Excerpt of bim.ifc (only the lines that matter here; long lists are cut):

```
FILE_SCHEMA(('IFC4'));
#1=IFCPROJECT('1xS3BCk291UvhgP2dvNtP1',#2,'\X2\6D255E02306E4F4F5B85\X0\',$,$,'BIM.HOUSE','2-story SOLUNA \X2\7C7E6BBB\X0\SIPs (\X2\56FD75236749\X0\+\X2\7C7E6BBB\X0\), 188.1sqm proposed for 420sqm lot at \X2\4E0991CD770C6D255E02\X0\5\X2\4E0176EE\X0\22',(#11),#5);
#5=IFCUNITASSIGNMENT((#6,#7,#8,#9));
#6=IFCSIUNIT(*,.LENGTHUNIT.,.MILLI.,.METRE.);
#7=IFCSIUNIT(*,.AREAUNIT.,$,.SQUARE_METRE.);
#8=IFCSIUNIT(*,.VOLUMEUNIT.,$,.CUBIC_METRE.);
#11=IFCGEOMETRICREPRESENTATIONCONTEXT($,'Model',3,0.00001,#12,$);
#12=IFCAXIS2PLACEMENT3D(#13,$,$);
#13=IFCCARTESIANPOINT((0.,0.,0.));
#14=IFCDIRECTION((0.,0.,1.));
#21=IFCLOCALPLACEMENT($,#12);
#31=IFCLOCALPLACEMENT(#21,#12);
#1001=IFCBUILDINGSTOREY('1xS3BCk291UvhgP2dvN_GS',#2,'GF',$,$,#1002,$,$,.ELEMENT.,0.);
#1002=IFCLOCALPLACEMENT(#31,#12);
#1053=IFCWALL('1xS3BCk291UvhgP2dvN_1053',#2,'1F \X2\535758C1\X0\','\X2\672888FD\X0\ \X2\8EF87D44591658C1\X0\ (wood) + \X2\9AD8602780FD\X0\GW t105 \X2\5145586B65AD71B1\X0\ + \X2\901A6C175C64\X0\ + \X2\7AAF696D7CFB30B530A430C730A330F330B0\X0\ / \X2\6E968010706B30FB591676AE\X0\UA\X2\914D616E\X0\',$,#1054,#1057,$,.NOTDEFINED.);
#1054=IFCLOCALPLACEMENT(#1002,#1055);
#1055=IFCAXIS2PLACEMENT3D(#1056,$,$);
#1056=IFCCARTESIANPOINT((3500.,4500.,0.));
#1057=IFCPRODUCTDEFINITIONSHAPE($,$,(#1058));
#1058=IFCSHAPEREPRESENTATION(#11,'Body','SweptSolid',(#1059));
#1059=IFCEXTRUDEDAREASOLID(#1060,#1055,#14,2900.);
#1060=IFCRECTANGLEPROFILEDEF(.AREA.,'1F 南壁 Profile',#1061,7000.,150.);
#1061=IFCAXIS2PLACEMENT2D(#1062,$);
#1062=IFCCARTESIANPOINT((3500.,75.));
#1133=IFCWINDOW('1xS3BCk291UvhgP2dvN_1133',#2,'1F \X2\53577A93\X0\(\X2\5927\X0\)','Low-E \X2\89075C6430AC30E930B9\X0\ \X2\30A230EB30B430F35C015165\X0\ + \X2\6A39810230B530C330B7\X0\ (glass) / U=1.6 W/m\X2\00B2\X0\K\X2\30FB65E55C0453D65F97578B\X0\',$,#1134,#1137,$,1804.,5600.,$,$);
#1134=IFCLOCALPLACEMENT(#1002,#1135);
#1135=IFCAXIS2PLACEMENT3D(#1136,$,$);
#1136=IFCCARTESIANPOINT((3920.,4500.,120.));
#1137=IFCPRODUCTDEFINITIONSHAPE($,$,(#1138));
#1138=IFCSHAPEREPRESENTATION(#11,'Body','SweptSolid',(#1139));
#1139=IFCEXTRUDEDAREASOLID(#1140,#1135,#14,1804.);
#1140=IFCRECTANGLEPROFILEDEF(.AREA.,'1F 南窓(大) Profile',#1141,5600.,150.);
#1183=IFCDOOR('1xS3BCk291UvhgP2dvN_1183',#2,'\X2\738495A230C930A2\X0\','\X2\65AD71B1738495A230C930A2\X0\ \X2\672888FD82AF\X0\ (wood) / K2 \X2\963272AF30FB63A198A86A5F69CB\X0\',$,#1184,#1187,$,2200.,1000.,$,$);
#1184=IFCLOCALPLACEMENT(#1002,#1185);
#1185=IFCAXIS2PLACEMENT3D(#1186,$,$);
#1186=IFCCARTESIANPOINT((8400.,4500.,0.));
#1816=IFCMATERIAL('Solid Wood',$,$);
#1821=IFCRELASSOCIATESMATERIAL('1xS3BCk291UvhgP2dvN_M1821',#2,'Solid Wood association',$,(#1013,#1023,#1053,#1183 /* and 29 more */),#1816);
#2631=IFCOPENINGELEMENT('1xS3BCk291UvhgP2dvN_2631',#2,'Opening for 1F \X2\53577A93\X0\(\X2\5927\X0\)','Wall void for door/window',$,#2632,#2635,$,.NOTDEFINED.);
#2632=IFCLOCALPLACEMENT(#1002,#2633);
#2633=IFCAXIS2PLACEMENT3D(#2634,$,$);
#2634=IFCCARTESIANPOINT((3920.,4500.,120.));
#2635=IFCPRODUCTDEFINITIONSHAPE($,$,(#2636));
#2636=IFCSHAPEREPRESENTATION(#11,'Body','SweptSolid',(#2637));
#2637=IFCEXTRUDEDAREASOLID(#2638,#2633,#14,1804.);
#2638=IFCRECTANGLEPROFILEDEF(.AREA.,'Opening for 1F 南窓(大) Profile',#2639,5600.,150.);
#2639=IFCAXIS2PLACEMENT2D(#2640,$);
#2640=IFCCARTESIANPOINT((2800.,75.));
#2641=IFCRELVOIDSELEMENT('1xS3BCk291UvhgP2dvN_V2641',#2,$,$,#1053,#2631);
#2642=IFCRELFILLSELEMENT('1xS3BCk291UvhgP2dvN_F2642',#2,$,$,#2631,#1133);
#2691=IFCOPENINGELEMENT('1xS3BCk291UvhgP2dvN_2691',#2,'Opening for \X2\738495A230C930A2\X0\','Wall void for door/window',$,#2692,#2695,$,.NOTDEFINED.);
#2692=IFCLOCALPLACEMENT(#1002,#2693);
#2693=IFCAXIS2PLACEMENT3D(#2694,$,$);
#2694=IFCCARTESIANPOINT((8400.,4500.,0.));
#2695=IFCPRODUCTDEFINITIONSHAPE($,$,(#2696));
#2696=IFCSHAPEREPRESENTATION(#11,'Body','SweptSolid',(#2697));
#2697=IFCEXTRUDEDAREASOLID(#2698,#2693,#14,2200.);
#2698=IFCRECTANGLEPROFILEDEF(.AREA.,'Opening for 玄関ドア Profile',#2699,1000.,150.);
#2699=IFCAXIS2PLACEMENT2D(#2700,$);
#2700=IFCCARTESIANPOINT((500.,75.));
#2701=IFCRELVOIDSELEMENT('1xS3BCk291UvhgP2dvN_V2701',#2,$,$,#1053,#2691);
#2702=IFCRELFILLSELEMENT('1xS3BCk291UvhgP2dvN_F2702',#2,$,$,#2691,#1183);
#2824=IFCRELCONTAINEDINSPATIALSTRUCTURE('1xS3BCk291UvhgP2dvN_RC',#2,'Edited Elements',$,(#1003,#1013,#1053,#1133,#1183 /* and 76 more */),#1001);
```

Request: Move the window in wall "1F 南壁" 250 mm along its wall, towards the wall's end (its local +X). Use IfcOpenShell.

```python
import ifcopenshell
import ifcopenshell.api.geometry
import ifcopenshell.util.placement

model = ifcopenshell.open("bim.ifc")

window = model.by_id(1133)
opening = window.FillsVoids[0].RelatingOpeningElement
wall = opening.VoidsElements[0].RelatingBuildingElement

wall_matrix = ifcopenshell.util.placement.get_local_placement(wall.ObjectPlacement)
shift = wall_matrix[:3, 0] * 250.0
before = ifcopenshell.util.placement.get_local_placement(window.ObjectPlacement)[:3, 3].copy()

# The window is not placed relative to its opening, so move both.
for product in (opening, window):
    matrix = ifcopenshell.util.placement.get_local_placement(product.ObjectPlacement)
    matrix[:3, 3] += shift
    ifcopenshell.api.geometry.edit_object_placement(model, product=product, matrix=matrix, is_si=False)

after = ifcopenshell.util.placement.get_local_placement(window.ObjectPlacement)[:3, 3]
print("window moved by", (after - before).round(3) + 0.0)

model.write("bim-out.ifc")
```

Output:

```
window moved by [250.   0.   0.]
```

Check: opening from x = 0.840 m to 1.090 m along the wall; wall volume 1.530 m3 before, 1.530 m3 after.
